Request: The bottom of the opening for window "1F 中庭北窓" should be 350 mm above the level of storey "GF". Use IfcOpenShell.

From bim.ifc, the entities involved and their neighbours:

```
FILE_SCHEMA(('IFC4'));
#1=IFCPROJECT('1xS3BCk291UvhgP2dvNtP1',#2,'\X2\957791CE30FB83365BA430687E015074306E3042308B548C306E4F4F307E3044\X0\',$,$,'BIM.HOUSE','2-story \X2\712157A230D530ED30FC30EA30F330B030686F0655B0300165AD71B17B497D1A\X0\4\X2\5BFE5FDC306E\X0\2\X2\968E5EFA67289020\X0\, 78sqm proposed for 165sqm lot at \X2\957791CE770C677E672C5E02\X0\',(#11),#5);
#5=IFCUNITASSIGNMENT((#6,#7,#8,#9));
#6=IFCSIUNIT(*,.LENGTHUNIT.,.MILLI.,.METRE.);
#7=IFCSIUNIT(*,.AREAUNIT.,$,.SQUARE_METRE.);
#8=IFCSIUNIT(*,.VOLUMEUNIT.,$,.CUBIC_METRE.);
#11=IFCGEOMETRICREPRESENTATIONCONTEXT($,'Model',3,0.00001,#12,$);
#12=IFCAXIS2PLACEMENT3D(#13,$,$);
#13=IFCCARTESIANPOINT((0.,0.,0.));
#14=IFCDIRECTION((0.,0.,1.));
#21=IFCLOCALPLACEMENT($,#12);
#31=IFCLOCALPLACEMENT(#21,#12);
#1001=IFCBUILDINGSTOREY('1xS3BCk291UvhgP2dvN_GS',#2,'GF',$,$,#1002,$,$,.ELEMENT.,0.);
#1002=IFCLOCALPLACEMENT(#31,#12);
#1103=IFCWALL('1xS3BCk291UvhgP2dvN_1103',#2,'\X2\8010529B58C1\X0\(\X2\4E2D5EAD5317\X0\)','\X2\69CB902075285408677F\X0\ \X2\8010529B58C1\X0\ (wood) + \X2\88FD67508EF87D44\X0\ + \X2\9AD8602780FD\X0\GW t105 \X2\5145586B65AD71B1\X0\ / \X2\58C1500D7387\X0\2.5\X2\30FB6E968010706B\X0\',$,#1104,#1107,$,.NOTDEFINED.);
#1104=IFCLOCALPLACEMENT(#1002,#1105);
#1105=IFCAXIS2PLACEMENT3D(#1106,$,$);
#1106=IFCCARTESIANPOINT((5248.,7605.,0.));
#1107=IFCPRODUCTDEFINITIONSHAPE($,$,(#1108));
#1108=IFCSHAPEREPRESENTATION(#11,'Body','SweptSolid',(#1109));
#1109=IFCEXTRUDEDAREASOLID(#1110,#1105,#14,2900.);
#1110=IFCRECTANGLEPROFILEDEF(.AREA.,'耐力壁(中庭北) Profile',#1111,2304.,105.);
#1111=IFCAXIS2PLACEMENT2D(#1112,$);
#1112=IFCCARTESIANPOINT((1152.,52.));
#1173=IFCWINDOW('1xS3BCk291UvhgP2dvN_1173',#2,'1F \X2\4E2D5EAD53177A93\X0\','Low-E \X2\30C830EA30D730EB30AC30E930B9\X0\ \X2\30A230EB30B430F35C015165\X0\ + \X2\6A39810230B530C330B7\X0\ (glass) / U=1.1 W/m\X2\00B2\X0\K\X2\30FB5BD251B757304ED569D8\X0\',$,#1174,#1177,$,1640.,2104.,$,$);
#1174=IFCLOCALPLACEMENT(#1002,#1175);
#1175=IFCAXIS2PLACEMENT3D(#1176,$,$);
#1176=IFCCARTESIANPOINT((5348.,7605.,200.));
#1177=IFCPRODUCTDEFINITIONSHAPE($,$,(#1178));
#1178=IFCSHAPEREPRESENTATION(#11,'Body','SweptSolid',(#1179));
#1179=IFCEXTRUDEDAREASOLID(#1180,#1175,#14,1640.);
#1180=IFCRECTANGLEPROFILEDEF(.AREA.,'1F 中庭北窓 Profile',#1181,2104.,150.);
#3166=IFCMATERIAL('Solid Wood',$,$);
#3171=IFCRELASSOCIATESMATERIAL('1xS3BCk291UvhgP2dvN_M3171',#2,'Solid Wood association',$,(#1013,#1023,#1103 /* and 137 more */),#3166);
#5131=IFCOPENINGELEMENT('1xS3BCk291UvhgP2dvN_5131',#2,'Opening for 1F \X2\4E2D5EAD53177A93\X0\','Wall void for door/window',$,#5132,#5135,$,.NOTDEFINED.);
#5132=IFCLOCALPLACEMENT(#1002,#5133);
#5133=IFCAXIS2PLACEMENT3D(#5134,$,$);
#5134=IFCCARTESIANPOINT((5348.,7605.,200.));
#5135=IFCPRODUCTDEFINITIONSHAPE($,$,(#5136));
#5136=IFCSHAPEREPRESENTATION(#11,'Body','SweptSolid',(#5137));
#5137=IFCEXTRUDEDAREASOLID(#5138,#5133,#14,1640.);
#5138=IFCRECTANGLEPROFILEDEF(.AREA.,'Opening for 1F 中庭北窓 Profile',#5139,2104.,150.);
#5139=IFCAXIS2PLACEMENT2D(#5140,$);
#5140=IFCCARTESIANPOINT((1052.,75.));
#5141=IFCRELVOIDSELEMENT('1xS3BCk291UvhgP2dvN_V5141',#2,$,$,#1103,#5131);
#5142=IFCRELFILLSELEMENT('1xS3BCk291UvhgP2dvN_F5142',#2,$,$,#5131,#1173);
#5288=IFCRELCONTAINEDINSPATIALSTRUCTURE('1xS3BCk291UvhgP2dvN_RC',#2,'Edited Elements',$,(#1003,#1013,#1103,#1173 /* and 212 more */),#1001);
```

```python
import numpy as np
import ifcopenshell
import ifcopenshell.api.geometry
import ifcopenshell.geom
import ifcopenshell.util.element
import ifcopenshell.util.placement
import ifcopenshell.util.shape
import ifcopenshell.util.unit

model = ifcopenshell.open("bim.ifc")
unit_scale = ifcopenshell.util.unit.calculate_unit_scale(model)

window = model.by_id(1173)
opening = window.FillsVoids[0].RelatingOpeningElement
storey = ifcopenshell.util.element.get_container(window, ifc_class="IfcBuildingStorey")
level = ifcopenshell.util.placement.get_local_placement(storey.ObjectPlacement)[2, 3]

# The opening's origin need not be at the sill, so measure its lowest point.
shape = ifcopenshell.geom.create_shape(ifcopenshell.geom.settings(), opening)
bottom = ifcopenshell.util.shape.get_shape_bottom_elevation(shape, shape.geometry) / unit_scale
dz = level + 350.0 - bottom

shift = np.array([0.0, 0.0, dz])
# The window is not placed relative to its opening, so move both.
for product in (opening, window):
    matrix = ifcopenshell.util.placement.get_local_placement(product.ObjectPlacement)
    matrix[:3, 3] += shift
    ifcopenshell.api.geometry.edit_object_placement(model, product=product, matrix=matrix, is_si=False)

print(f"moved by {dz * unit_scale:+.3f} m")

model.write("bim_v2.ifc")
```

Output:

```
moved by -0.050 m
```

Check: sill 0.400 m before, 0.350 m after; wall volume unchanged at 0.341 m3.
